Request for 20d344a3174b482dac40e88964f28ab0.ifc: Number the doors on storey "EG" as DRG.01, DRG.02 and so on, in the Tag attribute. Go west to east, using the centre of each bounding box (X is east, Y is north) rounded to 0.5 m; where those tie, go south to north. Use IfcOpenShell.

First a look at what the model holds.

```python
import ifcopenshell
import ifcopenshell.util.element
import ifcopenshell.util.placement

model = ifcopenshell.open("20d344a3174b482dac40e88964f28ab0.ifc")
print(model.schema)
storey = next(s for s in model.by_type("IfcBuildingStorey") if s.Name == "EG")
doors = [e for e in ifcopenshell.util.element.get_decomposition(storey) if e.is_a("IfcDoor")]
for e in sorted(doors, key=lambda e: e.id()):
    origin = ifcopenshell.util.placement.get_local_placement(e.ObjectPlacement)[:3, 3]
    print(e.id(), e.Tag, e.Name, origin.round(2) + 0.0, sep=" | ")
```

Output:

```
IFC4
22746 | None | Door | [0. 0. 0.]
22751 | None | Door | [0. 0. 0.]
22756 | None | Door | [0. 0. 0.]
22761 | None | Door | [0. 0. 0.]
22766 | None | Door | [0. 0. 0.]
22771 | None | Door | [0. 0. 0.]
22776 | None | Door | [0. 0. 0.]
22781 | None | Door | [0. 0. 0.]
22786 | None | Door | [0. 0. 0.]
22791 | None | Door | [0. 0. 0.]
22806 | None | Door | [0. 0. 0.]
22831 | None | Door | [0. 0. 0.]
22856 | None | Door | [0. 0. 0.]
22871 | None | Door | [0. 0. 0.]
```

```python
import ifcopenshell
import ifcopenshell.geom
import ifcopenshell.util.element
import ifcopenshell.util.shape

model = ifcopenshell.open("20d344a3174b482dac40e88964f28ab0.ifc")
settings = ifcopenshell.geom.settings()
settings.set("use-world-coords", True)


def centre(element):
    shape = ifcopenshell.geom.create_shape(settings, element)
    return ifcopenshell.util.shape.get_bbox_centroid(shape.geometry)


storey = next(s for s in model.by_type("IfcBuildingStorey") if s.Name == "EG")
doors = [e for e in ifcopenshell.util.element.get_decomposition(storey) if e.is_a("IfcDoor")]

# Insertion points can sit at a corner or the storey origin, so sort by the geometry (in metres).
centres = {e: centre(e) for e in doors}
doors.sort(key=lambda e: (round(centres[e][0] / 0.5), centres[e][1]))

for i, e in enumerate(doors, start=1):
    number = f"DRG.{i:02d}"
    e.Tag = number
    print(e.id(), number)

model.write("20d344a3174b482dac40e88964f28ab0_v2.ifc")
```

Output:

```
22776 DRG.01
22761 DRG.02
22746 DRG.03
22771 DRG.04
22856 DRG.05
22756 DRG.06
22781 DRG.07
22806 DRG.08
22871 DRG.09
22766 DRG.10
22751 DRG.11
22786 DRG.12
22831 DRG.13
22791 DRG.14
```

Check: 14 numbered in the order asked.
